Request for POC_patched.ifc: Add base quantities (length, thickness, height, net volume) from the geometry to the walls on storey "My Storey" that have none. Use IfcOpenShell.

First a look at what the model holds.

```python
import ifcopenshell
import ifcopenshell.util.element
import ifcopenshell.util.unit

model = ifcopenshell.open("POC_patched.ifc")
print(model.schema)
for unit_type in ("LENGTHUNIT", "AREAUNIT", "VOLUMEUNIT"):
    print(unit_type, ifcopenshell.util.unit.calculate_unit_scale(model, unit_type))
storey = next(s for s in model.by_type("IfcBuildingStorey") if s.Name == "My Storey")
walls = [e for e in ifcopenshell.util.element.get_decomposition(storey) if e.is_a("IfcWall")]
for e in sorted(walls, key=lambda e: e.id()):
    print(e.id(), e.is_a(), e.Name, list(ifcopenshell.util.element.get_psets(e, qtos_only=True)), sep=" | ")
```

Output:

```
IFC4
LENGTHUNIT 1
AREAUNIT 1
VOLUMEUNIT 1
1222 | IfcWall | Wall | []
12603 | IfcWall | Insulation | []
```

```python
import ifcopenshell
import ifcopenshell.api.pset
import ifcopenshell.geom
import ifcopenshell.util.element
import ifcopenshell.util.shape
import ifcopenshell.util.unit

model = ifcopenshell.open("POC_patched.ifc")
unit_scale = ifcopenshell.util.unit.calculate_unit_scale(model)
volume_scale = ifcopenshell.util.unit.calculate_unit_scale(model, "VOLUMEUNIT")
settings = ifcopenshell.geom.settings()

storey = next(s for s in model.by_type("IfcBuildingStorey") if s.Name == "My Storey")
walls = [e for e in ifcopenshell.util.element.get_decomposition(storey) if e.is_a("IfcWall")]

for e in sorted(walls, key=lambda e: e.id()):
    if ifcopenshell.util.element.get_psets(e, qtos_only=True, should_inherit=False):
        continue
    # Geometry comes back in metres, in the element's own axes.
    shape = ifcopenshell.geom.create_shape(settings, e)
    values = {
        "Length": ifcopenshell.util.shape.get_x(shape.geometry) / unit_scale,
        "Width": ifcopenshell.util.shape.get_y(shape.geometry) / unit_scale,
        "Height": ifcopenshell.util.shape.get_z(shape.geometry) / unit_scale,
        "NetVolume": ifcopenshell.util.shape.get_volume(shape.geometry) / volume_scale,
    }
    qto = ifcopenshell.api.pset.add_qto(model, product=e, name="Qto_WallBaseQuantities")
    ifcopenshell.api.pset.edit_qto(model, qto=qto, properties=values)
    print(e.id(), {k: round(v, 3) for k, v in values.items()})

model.write("POC_patched_edited.ifc")
```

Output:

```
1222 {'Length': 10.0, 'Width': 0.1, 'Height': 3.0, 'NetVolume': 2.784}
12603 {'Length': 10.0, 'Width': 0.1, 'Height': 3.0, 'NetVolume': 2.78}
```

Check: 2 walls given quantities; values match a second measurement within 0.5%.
